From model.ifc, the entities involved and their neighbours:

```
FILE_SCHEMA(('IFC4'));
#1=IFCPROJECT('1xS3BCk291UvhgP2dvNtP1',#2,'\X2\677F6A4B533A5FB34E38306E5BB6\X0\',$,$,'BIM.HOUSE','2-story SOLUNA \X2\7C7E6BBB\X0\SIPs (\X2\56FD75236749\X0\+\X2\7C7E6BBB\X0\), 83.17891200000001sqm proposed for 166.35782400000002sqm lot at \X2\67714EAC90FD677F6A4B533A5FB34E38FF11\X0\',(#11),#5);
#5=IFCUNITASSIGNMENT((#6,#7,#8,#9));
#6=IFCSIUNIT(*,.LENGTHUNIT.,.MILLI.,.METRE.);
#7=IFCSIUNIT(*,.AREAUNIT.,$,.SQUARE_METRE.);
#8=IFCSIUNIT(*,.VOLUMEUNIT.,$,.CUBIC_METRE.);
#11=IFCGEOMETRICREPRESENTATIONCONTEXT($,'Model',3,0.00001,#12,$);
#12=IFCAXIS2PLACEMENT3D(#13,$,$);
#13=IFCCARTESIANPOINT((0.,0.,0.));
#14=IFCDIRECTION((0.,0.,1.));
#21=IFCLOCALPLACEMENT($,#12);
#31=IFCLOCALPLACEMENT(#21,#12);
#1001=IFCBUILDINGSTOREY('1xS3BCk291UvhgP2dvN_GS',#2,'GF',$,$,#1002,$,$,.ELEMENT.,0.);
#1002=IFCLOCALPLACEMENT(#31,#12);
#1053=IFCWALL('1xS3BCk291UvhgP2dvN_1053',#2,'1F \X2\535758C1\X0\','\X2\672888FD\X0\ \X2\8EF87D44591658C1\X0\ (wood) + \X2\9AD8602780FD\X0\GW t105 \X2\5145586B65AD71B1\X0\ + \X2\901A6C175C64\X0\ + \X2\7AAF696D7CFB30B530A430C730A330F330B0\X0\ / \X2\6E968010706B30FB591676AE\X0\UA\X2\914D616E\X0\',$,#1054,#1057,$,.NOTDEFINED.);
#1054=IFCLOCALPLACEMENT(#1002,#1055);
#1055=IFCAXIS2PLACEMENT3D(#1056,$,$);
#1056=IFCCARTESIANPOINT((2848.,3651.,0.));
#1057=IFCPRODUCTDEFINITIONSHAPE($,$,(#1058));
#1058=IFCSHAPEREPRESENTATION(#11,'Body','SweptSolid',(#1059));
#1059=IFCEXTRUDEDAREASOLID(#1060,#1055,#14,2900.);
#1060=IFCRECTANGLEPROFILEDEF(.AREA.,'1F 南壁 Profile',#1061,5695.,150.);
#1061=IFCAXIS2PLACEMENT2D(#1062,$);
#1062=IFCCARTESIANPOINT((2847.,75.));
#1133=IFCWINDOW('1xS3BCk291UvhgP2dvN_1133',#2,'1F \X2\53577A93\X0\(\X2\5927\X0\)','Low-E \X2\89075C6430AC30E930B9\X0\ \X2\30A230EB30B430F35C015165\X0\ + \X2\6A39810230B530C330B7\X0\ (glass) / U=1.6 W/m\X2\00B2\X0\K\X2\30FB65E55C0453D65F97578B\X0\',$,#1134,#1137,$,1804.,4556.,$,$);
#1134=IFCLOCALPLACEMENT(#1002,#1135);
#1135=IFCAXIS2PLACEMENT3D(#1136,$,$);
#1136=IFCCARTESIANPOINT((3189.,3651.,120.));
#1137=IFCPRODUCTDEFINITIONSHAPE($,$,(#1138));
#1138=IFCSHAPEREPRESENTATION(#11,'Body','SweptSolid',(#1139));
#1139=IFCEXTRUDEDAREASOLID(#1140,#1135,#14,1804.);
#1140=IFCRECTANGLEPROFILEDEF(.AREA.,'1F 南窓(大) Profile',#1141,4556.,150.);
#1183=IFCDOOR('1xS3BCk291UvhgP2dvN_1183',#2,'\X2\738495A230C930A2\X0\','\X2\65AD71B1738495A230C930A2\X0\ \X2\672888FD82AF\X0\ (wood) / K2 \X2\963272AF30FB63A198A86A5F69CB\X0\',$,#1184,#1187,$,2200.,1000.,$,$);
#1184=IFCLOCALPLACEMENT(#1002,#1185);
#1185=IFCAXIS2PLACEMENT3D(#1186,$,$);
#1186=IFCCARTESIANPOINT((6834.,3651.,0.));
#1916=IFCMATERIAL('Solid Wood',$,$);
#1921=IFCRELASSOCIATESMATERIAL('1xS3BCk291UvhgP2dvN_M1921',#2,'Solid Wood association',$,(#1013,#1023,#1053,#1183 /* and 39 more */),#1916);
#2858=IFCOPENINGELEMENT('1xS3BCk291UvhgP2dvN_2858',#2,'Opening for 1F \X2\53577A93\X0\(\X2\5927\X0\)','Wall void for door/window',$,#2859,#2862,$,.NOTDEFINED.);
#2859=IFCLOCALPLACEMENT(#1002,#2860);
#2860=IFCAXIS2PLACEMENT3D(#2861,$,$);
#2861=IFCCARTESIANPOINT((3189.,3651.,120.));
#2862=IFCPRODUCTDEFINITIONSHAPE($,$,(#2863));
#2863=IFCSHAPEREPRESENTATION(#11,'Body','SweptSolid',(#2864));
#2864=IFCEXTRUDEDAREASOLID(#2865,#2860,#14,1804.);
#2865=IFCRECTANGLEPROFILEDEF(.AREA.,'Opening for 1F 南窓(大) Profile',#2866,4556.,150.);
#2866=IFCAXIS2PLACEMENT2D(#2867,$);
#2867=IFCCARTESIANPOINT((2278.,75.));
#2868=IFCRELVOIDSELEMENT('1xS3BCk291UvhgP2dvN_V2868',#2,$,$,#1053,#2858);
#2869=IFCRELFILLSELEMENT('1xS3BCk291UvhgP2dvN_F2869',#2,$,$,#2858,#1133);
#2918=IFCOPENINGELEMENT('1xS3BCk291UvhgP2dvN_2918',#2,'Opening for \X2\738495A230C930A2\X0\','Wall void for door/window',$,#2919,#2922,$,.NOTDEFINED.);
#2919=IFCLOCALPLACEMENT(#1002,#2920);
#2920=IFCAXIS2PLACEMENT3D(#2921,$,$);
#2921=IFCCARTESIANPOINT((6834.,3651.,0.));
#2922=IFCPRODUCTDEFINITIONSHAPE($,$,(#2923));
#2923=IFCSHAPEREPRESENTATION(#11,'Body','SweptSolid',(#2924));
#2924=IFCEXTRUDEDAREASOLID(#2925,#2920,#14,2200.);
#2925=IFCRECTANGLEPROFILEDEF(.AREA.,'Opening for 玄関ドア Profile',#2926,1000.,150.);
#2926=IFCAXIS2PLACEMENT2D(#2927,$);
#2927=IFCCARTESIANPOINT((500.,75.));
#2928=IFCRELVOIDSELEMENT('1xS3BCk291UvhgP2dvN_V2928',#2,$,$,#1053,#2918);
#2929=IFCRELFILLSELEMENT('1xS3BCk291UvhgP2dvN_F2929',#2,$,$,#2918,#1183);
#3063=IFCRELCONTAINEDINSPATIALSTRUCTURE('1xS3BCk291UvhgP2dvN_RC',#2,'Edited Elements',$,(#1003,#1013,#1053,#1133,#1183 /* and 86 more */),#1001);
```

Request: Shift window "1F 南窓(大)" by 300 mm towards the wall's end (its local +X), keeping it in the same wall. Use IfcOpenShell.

```python
import ifcopenshell
import ifcopenshell.api.geometry
import ifcopenshell.util.placement
import ifcopenshell.util.unit

model = ifcopenshell.open("model.ifc")
unit_scale = ifcopenshell.util.unit.calculate_unit_scale(model)

window = model.by_id(1133)
opening = window.FillsVoids[0].RelatingOpeningElement
wall = opening.VoidsElements[0].RelatingBuildingElement

wall_matrix = ifcopenshell.util.placement.get_local_placement(wall.ObjectPlacement)
shift = wall_matrix[:3, 0] * 0.3 / unit_scale
before = ifcopenshell.util.placement.get_local_placement(window.ObjectPlacement)[:3, 3].copy()

# The window is not placed relative to its opening, so move both.
for product in (opening, window):
    matrix = ifcopenshell.util.placement.get_local_placement(product.ObjectPlacement)
    matrix[:3, 3] += shift
    ifcopenshell.api.geometry.edit_object_placement(model, product=product, matrix=matrix, is_si=False)

after = ifcopenshell.util.placement.get_local_placement(window.ObjectPlacement)[:3, 3]
print("window moved by", (after - before).round(3) + 0.0)

model.write("model-out.ifc")
```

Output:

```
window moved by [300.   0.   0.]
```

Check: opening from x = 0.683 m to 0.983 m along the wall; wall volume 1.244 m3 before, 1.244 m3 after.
